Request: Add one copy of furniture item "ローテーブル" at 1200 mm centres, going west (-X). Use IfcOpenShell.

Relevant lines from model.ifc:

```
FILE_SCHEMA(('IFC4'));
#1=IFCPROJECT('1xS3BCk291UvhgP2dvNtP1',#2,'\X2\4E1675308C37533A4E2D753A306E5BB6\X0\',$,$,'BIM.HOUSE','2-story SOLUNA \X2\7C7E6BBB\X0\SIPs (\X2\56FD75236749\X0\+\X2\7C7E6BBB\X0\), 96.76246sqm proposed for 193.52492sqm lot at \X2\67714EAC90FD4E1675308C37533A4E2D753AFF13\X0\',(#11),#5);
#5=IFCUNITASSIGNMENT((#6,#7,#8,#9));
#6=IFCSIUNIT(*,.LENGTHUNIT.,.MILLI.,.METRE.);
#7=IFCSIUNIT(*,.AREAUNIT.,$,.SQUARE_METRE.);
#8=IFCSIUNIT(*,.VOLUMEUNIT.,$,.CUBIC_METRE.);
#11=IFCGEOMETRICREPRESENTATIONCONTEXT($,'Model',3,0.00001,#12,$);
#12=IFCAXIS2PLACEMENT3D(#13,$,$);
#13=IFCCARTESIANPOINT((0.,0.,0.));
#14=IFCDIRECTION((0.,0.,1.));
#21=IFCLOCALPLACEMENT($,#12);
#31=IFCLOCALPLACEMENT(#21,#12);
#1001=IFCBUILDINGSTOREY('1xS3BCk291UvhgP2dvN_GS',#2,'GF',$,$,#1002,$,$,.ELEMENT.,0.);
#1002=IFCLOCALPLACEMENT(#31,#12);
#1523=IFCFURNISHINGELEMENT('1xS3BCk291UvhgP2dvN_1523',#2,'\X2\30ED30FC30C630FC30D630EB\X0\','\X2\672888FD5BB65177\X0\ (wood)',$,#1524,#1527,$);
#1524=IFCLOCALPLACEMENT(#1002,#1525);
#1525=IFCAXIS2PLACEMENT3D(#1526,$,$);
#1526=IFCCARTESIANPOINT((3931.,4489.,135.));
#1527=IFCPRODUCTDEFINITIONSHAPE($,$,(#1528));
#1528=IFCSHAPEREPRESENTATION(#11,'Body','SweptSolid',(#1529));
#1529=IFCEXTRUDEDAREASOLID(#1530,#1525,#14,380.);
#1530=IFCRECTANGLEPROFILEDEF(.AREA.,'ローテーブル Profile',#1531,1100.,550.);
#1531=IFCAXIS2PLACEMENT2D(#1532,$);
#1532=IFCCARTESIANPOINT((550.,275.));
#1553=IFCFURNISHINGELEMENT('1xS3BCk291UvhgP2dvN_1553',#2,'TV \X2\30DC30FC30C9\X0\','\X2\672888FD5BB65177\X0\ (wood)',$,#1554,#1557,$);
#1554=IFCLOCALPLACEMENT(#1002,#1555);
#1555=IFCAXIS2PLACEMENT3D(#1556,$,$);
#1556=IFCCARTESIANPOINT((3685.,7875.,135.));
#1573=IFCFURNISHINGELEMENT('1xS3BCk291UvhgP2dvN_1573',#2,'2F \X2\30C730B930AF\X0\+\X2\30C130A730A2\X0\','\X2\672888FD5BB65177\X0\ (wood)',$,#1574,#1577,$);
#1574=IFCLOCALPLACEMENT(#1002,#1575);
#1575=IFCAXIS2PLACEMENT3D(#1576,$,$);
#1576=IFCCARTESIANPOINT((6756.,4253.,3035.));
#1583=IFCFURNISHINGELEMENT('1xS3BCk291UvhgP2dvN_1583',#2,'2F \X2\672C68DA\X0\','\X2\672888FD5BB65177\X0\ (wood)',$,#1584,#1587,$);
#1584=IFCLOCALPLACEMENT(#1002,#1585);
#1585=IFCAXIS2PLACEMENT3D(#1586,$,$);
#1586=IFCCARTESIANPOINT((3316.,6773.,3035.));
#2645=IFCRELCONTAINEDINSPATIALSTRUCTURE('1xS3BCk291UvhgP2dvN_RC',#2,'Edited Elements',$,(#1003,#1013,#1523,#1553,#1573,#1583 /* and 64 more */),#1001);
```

```python
import numpy as np
import ifcopenshell
import ifcopenshell.api.geometry
import ifcopenshell.api.root
import ifcopenshell.util.element
import ifcopenshell.util.placement
import ifcopenshell.util.unit

model = ifcopenshell.open("model.ifc")
unit_scale = ifcopenshell.util.unit.calculate_unit_scale(model)


def reuse_history(source, copy):
    """copy_class also copies each property set's owner history, people and application; keep the originals."""
    for rel in copy.IsDefinedBy:
        if rel.is_a("IfcRelDefinesByProperties") and (history := rel.RelatingPropertyDefinition.OwnerHistory):
            rel.RelatingPropertyDefinition.OwnerHistory = source.OwnerHistory
            ifcopenshell.util.element.remove_deep2(model, history)


source = model.by_guid("1xS3BCk291UvhgP2dvN_1523")
base = ifcopenshell.util.placement.get_local_placement(source.ObjectPlacement)
step = np.array([-1.0, 0.0, 0.0]) * 1.2 / unit_scale

for i in range(1, 2):
    copy = ifcopenshell.api.root.copy_class(model, product=source)
    copy.Representation = ifcopenshell.util.element.copy_deep(
        model, source.Representation, exclude=["IfcGeometricRepresentationContext", "IfcRepresentationMap"]
    )
    reuse_history(source, copy)
    matrix = base.copy()
    matrix[:3, 3] += i * step
    print("added at", matrix[:3, 3].round(3) + 0.0)
    ifcopenshell.api.geometry.edit_object_placement(model, product=copy, matrix=matrix, is_si=False)

model.write("model-out.ifc")
```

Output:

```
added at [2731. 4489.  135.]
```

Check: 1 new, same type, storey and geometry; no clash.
